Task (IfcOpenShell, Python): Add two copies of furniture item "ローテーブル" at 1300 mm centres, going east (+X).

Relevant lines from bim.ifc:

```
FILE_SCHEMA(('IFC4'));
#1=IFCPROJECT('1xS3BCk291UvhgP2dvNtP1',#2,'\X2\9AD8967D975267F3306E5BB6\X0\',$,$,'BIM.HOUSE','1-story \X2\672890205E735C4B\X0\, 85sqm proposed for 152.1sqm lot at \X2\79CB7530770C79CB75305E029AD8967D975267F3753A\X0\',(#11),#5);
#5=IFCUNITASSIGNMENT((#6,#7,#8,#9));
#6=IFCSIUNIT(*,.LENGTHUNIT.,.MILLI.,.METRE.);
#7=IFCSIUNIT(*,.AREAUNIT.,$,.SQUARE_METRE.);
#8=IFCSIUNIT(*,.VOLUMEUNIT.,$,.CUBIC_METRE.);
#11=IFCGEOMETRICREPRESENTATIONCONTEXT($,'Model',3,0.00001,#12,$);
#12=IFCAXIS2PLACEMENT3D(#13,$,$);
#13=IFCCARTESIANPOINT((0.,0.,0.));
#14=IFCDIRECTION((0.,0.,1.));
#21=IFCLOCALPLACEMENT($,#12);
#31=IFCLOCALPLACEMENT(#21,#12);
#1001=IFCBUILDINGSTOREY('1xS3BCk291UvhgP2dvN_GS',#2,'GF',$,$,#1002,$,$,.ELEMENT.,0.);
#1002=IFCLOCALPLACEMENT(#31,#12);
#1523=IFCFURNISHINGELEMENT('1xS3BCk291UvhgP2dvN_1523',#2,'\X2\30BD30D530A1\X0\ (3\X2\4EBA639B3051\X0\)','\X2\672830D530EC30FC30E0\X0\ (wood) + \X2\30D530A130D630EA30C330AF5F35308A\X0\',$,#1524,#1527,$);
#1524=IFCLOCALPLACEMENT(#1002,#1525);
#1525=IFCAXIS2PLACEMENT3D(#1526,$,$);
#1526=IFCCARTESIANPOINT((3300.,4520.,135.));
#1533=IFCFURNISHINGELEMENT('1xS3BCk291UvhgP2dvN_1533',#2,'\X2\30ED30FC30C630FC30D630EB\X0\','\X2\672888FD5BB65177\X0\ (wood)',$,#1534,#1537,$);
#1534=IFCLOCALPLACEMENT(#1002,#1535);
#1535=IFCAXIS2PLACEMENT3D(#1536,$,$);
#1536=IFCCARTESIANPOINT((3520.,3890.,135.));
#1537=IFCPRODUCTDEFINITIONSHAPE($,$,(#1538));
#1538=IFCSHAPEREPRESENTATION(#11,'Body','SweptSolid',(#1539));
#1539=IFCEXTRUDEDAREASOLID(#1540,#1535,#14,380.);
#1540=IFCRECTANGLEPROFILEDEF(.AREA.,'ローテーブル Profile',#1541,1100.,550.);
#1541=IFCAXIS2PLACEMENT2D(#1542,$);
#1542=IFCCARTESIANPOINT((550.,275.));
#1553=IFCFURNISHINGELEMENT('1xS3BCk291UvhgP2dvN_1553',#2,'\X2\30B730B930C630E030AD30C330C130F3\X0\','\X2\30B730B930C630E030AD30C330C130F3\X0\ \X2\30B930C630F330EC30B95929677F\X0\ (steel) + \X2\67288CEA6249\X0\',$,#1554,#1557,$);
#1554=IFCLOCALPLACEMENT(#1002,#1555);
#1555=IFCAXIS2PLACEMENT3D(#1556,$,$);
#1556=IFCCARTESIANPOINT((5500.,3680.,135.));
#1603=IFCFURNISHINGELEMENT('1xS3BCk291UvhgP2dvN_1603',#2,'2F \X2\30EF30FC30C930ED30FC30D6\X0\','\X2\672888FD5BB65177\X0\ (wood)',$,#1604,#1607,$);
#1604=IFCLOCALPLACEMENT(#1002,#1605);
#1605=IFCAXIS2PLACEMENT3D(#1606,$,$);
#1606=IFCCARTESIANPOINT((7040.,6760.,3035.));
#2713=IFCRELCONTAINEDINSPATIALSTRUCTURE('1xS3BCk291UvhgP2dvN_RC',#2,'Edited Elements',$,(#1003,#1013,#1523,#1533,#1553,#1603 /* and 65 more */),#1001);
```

```python
import numpy as np
import ifcopenshell
import ifcopenshell.api.geometry
import ifcopenshell.api.root
import ifcopenshell.util.element
import ifcopenshell.util.placement
import ifcopenshell.util.unit

model = ifcopenshell.open("bim.ifc")
unit_scale = ifcopenshell.util.unit.calculate_unit_scale(model)


def reuse_history(source, copy):
    """copy_class also copies each property set's owner history, people and application; keep the originals."""
    for rel in copy.IsDefinedBy:
        if rel.is_a("IfcRelDefinesByProperties") and (history := rel.RelatingPropertyDefinition.OwnerHistory):
            rel.RelatingPropertyDefinition.OwnerHistory = source.OwnerHistory
            ifcopenshell.util.element.remove_deep2(model, history)


source = model.by_guid("1xS3BCk291UvhgP2dvN_1533")
base = ifcopenshell.util.placement.get_local_placement(source.ObjectPlacement)
step = np.array([1.0, 0.0, 0.0]) * 1.3 / unit_scale

for i in range(1, 3):
    copy = ifcopenshell.api.root.copy_class(model, product=source)
    copy.Representation = ifcopenshell.util.element.copy_deep(
        model, source.Representation, exclude=["IfcGeometricRepresentationContext", "IfcRepresentationMap"]
    )
    reuse_history(source, copy)
    matrix = base.copy()
    matrix[:3, 3] += i * step
    print("added at", matrix[:3, 3].round(3) + 0.0)
    ifcopenshell.api.geometry.edit_object_placement(model, product=copy, matrix=matrix, is_si=False)

model.write("bim_updated.ifc")
```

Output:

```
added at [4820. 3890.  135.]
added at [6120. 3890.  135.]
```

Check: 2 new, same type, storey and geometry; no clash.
